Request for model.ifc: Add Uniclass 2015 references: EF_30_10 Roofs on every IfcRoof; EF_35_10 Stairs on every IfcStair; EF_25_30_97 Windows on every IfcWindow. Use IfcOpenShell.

First a look at what the model holds.

```python
import ifcopenshell

model = ifcopenshell.open("model.ifc")
print(model.schema)
print("classifications:", [c.Name for c in model.by_type("IfcClassification")])
for ifc_class in ("IfcDoor", "IfcRoof", "IfcStair", "IfcWall", "IfcWindow"):
    print(ifc_class, len(model.by_type(ifc_class)))
```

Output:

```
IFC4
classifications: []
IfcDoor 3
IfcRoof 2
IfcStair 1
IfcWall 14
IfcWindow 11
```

```python
import ifcopenshell
import ifcopenshell.api.classification

model = ifcopenshell.open("model.ifc")

system = ifcopenshell.api.classification.add_classification(model, classification="Uniclass 2015")

codes = {
    "IfcRoof": ("EF_30_10", "Roofs"),
    "IfcStair": ("EF_35_10", "Stairs"),
    "IfcWindow": ("EF_25_30_97", "Windows"),
}
for ifc_class, (code, name) in codes.items():
    products = model.by_type(ifc_class)
    ifcopenshell.api.classification.add_reference(
        model, products=products, classification=system, identification=code, name=name
    )
    print(code, len(products))

model.write("model_updated.ifc")
```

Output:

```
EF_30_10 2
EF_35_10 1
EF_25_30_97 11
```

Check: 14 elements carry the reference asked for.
